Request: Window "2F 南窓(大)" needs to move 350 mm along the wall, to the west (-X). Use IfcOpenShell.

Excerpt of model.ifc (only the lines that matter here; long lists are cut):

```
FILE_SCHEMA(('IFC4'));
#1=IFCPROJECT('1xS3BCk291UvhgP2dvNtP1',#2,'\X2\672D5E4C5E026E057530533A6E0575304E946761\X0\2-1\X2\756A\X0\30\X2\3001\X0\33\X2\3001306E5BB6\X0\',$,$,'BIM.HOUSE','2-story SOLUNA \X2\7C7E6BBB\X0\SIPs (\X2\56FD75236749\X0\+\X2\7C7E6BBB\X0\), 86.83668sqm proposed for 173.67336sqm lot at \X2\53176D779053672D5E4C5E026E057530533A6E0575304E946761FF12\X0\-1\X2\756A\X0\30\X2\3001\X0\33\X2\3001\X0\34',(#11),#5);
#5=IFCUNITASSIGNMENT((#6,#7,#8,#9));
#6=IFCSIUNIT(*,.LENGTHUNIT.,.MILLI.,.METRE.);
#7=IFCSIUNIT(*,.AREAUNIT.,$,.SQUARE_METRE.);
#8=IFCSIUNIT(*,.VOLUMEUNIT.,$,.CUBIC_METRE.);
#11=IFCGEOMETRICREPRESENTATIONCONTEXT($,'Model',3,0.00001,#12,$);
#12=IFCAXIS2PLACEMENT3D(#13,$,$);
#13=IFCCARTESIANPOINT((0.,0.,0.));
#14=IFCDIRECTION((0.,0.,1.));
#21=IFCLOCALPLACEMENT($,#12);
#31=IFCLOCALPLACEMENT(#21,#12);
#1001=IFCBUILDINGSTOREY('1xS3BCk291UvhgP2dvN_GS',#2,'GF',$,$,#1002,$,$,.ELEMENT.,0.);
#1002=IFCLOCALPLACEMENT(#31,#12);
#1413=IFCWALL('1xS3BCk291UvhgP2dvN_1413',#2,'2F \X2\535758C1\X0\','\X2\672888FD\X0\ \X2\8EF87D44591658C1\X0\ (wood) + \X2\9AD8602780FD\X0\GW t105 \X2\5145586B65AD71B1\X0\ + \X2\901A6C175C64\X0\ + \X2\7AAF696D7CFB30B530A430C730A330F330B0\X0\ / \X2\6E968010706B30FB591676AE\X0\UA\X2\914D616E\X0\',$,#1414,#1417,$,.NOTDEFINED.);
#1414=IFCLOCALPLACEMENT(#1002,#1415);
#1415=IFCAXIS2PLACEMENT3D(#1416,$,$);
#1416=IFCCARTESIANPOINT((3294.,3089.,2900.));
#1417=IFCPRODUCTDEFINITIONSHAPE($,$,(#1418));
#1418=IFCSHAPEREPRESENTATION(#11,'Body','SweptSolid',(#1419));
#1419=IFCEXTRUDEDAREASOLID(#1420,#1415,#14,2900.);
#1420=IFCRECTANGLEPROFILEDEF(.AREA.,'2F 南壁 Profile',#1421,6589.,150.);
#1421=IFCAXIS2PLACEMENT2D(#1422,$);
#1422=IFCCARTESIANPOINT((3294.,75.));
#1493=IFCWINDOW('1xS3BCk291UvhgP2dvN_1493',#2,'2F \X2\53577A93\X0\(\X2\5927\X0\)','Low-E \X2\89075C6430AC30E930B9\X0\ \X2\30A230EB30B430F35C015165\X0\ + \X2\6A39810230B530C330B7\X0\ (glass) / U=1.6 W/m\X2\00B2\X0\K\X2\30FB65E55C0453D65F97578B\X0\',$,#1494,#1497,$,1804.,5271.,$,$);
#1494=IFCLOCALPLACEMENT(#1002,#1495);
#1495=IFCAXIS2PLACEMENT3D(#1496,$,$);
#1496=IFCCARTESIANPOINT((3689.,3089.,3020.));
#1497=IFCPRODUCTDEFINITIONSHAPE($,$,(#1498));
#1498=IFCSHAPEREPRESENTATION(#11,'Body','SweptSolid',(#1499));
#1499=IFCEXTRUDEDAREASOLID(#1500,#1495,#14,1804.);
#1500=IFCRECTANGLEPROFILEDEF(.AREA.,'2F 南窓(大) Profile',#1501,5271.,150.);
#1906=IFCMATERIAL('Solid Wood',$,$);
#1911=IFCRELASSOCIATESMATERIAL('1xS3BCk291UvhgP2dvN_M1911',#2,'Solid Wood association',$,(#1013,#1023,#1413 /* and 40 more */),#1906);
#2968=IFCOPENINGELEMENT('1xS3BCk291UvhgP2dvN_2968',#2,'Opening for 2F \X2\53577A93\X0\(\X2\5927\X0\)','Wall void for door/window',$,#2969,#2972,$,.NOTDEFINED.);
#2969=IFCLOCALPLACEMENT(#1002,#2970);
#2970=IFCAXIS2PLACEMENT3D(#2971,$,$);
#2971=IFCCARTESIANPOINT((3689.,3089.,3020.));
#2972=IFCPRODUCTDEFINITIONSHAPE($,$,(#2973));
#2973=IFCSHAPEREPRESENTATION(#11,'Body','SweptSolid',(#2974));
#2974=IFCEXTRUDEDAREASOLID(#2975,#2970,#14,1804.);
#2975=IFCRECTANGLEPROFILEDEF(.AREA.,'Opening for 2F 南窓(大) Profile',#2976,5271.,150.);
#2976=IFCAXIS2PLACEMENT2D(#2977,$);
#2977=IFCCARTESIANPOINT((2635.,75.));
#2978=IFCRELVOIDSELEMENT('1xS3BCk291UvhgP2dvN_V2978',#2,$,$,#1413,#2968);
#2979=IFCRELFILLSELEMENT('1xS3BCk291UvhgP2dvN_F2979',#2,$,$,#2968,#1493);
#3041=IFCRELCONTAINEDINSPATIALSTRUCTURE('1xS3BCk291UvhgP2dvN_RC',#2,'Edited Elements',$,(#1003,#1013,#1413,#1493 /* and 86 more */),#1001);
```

```python
import ifcopenshell
import ifcopenshell.api.geometry
import ifcopenshell.util.placement

model = ifcopenshell.open("model.ifc")

window = model.by_guid("1xS3BCk291UvhgP2dvN_1493")
opening = window.FillsVoids[0].RelatingOpeningElement
wall = opening.VoidsElements[0].RelatingBuildingElement

wall_matrix = ifcopenshell.util.placement.get_local_placement(wall.ObjectPlacement)
shift = wall_matrix[:3, 0] * -350.0
before = ifcopenshell.util.placement.get_local_placement(window.ObjectPlacement)[:3, 3].copy()

# The window is not placed relative to its opening, so move both.
for product in (opening, window):
    matrix = ifcopenshell.util.placement.get_local_placement(product.ObjectPlacement)
    matrix[:3, 3] += shift
    ifcopenshell.api.geometry.edit_object_placement(model, product=product, matrix=matrix, is_si=False)

after = ifcopenshell.util.placement.get_local_placement(window.ObjectPlacement)[:3, 3]
print("window moved by", (after - before).round(3) + 0.0)

model.write("model_rev.ifc")
```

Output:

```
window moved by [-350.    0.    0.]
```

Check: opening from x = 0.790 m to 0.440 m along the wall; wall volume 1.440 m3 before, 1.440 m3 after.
